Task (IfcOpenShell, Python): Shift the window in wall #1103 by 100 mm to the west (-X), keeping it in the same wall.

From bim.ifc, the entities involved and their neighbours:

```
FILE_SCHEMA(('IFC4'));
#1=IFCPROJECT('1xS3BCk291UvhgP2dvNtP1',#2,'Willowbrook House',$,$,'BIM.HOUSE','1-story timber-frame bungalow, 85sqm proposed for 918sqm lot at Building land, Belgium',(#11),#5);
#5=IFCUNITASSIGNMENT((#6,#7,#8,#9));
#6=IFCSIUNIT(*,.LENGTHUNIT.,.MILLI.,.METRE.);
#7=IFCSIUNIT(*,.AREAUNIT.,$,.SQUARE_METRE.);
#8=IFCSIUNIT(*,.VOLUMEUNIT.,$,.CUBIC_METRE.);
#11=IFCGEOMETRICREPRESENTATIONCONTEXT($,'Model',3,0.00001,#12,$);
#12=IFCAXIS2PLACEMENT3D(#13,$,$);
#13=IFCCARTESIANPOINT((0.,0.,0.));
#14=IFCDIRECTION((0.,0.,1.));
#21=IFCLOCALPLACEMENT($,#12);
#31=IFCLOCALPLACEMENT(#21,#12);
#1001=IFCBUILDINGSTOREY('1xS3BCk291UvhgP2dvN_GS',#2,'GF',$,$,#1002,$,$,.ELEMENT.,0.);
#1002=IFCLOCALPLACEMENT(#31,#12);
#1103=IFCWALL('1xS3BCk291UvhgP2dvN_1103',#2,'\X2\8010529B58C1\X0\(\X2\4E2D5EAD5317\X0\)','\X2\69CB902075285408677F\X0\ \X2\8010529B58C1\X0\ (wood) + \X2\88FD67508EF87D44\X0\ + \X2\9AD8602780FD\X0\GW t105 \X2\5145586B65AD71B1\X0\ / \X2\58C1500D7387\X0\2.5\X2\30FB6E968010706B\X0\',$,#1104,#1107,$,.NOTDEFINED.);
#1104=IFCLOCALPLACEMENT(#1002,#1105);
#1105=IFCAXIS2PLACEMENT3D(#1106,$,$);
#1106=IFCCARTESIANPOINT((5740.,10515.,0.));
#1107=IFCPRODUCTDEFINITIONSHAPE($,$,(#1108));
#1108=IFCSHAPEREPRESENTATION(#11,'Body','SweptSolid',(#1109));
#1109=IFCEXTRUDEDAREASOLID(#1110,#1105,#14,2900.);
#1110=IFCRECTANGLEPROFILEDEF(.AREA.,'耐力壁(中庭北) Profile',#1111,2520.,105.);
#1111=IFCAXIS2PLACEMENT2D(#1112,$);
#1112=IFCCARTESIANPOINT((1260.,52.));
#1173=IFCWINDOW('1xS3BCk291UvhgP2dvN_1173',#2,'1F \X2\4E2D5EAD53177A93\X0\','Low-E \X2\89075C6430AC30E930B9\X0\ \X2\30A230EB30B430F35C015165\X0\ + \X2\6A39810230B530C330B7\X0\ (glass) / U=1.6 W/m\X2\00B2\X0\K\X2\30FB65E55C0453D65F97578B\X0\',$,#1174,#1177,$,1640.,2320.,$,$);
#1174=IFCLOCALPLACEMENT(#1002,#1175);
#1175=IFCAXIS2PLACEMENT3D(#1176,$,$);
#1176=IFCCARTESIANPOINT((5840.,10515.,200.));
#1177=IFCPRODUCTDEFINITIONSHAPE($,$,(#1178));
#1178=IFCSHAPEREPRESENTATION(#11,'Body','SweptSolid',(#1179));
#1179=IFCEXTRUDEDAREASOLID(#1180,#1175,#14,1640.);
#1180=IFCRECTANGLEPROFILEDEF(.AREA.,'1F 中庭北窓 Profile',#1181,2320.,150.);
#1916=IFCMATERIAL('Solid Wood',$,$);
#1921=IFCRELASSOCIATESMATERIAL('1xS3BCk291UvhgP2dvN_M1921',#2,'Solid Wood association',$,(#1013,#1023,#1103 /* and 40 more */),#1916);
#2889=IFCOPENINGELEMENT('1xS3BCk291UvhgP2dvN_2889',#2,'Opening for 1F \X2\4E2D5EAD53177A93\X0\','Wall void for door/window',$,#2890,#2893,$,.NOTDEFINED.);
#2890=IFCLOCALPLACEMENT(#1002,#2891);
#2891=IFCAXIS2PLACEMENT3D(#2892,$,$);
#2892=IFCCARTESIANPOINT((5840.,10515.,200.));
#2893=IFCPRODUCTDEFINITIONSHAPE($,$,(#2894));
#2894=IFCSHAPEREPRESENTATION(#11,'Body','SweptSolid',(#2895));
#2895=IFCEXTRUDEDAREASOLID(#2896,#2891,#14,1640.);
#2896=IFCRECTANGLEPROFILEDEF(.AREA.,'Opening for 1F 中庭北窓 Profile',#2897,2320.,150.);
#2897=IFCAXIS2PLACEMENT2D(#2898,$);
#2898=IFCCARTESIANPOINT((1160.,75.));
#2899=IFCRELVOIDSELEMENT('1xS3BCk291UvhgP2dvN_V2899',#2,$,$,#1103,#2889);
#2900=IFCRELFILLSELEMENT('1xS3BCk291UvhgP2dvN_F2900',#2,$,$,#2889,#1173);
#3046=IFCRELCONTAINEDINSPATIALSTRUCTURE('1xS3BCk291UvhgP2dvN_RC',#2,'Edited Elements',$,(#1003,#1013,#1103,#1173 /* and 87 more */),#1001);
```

```python
import ifcopenshell
import ifcopenshell.api.geometry
import ifcopenshell.util.placement
import ifcopenshell.util.unit

model = ifcopenshell.open("bim.ifc")
unit_scale = ifcopenshell.util.unit.calculate_unit_scale(model)

window = model.by_guid("1xS3BCk291UvhgP2dvN_1173")
opening = window.FillsVoids[0].RelatingOpeningElement
wall = opening.VoidsElements[0].RelatingBuildingElement

wall_matrix = ifcopenshell.util.placement.get_local_placement(wall.ObjectPlacement)
shift = wall_matrix[:3, 0] * -0.1 / unit_scale
before = ifcopenshell.util.placement.get_local_placement(window.ObjectPlacement)[:3, 3].copy()

# The window is not placed relative to its opening, so move both.
for product in (opening, window):
    matrix = ifcopenshell.util.placement.get_local_placement(product.ObjectPlacement)
    matrix[:3, 3] += shift
    ifcopenshell.api.geometry.edit_object_placement(model, product=product, matrix=matrix, is_si=False)

after = ifcopenshell.util.placement.get_local_placement(window.ObjectPlacement)[:3, 3]
print("window moved by", (after - before).round(3) + 0.0)

model.write("bim_edited.ifc")
```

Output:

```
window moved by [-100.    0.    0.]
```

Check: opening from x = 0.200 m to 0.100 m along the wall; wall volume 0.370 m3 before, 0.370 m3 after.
